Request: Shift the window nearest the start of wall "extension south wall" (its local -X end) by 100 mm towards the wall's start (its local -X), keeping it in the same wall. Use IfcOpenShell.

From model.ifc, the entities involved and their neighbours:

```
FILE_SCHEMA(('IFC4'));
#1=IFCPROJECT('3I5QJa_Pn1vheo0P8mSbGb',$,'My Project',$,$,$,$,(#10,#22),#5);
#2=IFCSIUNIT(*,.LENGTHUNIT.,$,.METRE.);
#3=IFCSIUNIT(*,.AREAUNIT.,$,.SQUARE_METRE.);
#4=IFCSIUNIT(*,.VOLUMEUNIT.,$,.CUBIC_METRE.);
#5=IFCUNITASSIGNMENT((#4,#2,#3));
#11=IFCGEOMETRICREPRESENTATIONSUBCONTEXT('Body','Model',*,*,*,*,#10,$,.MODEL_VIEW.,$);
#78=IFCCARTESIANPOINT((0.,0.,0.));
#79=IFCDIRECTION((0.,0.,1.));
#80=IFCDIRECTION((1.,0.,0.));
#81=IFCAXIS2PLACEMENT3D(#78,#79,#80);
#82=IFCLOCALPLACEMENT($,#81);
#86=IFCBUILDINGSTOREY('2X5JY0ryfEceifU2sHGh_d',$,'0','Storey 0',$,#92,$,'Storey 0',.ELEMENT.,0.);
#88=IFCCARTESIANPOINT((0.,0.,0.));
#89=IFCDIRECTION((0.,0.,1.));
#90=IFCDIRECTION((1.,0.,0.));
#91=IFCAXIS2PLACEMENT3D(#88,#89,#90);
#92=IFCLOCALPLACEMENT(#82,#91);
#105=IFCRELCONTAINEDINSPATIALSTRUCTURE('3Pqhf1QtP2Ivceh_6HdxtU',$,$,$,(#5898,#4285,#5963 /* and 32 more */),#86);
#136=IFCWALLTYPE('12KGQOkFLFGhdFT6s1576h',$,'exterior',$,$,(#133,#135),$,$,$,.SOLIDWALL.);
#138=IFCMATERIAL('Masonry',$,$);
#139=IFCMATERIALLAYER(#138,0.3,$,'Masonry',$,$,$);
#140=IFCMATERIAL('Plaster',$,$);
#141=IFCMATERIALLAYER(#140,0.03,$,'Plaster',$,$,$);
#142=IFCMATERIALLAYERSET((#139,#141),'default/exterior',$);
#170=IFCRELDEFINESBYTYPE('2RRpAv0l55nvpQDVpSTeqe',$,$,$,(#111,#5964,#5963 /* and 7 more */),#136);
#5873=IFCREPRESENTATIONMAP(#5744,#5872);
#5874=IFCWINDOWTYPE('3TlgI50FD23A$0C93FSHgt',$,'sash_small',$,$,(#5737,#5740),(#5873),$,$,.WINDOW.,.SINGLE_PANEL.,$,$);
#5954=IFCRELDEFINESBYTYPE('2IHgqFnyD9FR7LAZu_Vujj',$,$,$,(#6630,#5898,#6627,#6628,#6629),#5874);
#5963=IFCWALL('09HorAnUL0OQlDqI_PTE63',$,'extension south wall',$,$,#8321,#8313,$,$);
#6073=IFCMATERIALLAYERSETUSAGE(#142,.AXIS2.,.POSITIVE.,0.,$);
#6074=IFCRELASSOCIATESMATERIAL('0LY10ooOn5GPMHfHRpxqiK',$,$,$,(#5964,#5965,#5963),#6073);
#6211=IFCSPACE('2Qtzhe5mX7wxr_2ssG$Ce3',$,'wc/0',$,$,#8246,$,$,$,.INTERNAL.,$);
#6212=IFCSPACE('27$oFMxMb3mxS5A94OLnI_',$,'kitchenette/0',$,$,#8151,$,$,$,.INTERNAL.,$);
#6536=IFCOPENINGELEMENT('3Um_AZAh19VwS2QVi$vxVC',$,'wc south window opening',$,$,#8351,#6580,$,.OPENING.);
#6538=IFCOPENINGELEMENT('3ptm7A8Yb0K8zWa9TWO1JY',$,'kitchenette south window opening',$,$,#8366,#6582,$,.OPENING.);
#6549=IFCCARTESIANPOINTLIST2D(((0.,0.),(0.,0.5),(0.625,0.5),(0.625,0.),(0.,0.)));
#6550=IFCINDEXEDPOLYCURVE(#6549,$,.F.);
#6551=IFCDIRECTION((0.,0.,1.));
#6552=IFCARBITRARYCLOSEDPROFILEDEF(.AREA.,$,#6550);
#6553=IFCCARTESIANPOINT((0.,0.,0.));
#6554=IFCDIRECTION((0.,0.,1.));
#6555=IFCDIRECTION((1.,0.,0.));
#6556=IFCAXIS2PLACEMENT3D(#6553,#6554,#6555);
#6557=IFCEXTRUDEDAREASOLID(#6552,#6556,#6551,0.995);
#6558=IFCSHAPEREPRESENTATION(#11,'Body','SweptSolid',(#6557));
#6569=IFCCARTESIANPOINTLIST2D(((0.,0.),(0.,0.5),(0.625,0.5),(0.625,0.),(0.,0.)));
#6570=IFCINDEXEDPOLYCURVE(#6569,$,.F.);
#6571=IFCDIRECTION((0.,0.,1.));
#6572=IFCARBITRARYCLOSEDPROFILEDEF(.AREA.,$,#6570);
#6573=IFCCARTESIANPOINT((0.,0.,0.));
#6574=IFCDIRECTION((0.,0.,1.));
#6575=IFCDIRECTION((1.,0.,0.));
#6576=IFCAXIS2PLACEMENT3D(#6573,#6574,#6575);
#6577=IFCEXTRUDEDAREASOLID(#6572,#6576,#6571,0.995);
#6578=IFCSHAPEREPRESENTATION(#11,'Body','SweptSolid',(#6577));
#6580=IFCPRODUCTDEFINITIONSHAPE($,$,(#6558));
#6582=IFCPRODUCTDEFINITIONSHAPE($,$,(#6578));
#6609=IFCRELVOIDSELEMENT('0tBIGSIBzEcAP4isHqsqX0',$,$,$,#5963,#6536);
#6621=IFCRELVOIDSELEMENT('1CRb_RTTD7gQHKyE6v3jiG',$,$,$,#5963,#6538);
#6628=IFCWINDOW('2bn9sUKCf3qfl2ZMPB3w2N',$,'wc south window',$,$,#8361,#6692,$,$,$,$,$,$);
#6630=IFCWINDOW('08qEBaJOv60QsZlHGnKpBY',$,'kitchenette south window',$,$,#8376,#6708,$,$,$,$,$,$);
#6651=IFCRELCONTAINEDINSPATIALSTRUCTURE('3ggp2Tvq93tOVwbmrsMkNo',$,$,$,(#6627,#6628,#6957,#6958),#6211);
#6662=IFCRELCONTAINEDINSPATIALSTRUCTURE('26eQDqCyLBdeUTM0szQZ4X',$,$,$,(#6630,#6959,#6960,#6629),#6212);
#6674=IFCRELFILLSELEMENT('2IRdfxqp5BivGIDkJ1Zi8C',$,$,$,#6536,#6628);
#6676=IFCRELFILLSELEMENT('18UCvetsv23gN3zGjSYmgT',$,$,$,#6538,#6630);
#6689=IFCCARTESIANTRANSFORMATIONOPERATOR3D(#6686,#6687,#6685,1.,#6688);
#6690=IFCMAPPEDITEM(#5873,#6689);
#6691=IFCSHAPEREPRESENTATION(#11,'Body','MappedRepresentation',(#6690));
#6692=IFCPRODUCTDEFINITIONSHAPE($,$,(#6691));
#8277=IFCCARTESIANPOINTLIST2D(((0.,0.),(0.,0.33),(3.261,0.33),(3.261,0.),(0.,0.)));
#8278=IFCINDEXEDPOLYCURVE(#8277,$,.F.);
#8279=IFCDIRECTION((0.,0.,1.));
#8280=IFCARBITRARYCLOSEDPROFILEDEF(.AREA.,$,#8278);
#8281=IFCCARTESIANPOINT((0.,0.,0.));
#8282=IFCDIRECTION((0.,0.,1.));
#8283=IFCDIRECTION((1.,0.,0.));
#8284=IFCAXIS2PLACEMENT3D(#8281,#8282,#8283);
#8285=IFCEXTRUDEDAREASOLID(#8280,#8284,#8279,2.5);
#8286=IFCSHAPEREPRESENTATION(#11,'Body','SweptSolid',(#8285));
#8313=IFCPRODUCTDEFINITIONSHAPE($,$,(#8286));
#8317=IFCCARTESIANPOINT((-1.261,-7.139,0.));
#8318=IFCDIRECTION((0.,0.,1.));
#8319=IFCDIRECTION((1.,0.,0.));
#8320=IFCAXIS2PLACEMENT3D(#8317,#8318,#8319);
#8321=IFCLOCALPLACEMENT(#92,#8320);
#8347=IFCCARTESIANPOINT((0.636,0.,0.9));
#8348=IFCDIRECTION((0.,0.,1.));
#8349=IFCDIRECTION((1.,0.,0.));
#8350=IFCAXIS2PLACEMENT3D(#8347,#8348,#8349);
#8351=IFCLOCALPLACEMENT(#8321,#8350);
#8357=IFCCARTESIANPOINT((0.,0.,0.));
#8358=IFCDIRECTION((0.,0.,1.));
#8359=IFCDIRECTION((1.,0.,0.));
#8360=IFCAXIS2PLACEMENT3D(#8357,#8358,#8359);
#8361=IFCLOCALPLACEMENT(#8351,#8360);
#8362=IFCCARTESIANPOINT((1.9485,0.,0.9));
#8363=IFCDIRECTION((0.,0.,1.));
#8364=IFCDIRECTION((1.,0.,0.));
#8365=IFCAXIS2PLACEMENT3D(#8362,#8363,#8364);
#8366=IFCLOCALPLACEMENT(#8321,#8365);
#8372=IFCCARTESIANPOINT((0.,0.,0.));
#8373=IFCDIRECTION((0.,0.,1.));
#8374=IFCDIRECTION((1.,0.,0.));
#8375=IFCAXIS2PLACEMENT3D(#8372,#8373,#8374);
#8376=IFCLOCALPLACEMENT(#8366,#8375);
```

```python
import ifcopenshell
import ifcopenshell.api.geometry
import ifcopenshell.util.placement
import ifcopenshell.util.unit

model = ifcopenshell.open("model.ifc")
unit_scale = ifcopenshell.util.unit.calculate_unit_scale(model)

window = model.by_guid("2bn9sUKCf3qfl2ZMPB3w2N")
opening = window.FillsVoids[0].RelatingOpeningElement
wall = opening.VoidsElements[0].RelatingBuildingElement

wall_matrix = ifcopenshell.util.placement.get_local_placement(wall.ObjectPlacement)
shift = wall_matrix[:3, 0] * -0.1 / unit_scale
before = ifcopenshell.util.placement.get_local_placement(window.ObjectPlacement)[:3, 3].copy()

# The window is placed relative to its opening, so it follows when the opening moves.
matrix = ifcopenshell.util.placement.get_local_placement(opening.ObjectPlacement)
matrix[:3, 3] += shift
ifcopenshell.api.geometry.edit_object_placement(
    model, product=opening, matrix=matrix, is_si=False, should_transform_children=True
)

after = ifcopenshell.util.placement.get_local_placement(window.ObjectPlacement)[:3, 3]
print("window moved by", (after - before).round(3) + 0.0)

model.write("model-out.ifc")
```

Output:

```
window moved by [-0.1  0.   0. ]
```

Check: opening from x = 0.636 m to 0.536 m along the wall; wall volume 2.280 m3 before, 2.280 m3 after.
